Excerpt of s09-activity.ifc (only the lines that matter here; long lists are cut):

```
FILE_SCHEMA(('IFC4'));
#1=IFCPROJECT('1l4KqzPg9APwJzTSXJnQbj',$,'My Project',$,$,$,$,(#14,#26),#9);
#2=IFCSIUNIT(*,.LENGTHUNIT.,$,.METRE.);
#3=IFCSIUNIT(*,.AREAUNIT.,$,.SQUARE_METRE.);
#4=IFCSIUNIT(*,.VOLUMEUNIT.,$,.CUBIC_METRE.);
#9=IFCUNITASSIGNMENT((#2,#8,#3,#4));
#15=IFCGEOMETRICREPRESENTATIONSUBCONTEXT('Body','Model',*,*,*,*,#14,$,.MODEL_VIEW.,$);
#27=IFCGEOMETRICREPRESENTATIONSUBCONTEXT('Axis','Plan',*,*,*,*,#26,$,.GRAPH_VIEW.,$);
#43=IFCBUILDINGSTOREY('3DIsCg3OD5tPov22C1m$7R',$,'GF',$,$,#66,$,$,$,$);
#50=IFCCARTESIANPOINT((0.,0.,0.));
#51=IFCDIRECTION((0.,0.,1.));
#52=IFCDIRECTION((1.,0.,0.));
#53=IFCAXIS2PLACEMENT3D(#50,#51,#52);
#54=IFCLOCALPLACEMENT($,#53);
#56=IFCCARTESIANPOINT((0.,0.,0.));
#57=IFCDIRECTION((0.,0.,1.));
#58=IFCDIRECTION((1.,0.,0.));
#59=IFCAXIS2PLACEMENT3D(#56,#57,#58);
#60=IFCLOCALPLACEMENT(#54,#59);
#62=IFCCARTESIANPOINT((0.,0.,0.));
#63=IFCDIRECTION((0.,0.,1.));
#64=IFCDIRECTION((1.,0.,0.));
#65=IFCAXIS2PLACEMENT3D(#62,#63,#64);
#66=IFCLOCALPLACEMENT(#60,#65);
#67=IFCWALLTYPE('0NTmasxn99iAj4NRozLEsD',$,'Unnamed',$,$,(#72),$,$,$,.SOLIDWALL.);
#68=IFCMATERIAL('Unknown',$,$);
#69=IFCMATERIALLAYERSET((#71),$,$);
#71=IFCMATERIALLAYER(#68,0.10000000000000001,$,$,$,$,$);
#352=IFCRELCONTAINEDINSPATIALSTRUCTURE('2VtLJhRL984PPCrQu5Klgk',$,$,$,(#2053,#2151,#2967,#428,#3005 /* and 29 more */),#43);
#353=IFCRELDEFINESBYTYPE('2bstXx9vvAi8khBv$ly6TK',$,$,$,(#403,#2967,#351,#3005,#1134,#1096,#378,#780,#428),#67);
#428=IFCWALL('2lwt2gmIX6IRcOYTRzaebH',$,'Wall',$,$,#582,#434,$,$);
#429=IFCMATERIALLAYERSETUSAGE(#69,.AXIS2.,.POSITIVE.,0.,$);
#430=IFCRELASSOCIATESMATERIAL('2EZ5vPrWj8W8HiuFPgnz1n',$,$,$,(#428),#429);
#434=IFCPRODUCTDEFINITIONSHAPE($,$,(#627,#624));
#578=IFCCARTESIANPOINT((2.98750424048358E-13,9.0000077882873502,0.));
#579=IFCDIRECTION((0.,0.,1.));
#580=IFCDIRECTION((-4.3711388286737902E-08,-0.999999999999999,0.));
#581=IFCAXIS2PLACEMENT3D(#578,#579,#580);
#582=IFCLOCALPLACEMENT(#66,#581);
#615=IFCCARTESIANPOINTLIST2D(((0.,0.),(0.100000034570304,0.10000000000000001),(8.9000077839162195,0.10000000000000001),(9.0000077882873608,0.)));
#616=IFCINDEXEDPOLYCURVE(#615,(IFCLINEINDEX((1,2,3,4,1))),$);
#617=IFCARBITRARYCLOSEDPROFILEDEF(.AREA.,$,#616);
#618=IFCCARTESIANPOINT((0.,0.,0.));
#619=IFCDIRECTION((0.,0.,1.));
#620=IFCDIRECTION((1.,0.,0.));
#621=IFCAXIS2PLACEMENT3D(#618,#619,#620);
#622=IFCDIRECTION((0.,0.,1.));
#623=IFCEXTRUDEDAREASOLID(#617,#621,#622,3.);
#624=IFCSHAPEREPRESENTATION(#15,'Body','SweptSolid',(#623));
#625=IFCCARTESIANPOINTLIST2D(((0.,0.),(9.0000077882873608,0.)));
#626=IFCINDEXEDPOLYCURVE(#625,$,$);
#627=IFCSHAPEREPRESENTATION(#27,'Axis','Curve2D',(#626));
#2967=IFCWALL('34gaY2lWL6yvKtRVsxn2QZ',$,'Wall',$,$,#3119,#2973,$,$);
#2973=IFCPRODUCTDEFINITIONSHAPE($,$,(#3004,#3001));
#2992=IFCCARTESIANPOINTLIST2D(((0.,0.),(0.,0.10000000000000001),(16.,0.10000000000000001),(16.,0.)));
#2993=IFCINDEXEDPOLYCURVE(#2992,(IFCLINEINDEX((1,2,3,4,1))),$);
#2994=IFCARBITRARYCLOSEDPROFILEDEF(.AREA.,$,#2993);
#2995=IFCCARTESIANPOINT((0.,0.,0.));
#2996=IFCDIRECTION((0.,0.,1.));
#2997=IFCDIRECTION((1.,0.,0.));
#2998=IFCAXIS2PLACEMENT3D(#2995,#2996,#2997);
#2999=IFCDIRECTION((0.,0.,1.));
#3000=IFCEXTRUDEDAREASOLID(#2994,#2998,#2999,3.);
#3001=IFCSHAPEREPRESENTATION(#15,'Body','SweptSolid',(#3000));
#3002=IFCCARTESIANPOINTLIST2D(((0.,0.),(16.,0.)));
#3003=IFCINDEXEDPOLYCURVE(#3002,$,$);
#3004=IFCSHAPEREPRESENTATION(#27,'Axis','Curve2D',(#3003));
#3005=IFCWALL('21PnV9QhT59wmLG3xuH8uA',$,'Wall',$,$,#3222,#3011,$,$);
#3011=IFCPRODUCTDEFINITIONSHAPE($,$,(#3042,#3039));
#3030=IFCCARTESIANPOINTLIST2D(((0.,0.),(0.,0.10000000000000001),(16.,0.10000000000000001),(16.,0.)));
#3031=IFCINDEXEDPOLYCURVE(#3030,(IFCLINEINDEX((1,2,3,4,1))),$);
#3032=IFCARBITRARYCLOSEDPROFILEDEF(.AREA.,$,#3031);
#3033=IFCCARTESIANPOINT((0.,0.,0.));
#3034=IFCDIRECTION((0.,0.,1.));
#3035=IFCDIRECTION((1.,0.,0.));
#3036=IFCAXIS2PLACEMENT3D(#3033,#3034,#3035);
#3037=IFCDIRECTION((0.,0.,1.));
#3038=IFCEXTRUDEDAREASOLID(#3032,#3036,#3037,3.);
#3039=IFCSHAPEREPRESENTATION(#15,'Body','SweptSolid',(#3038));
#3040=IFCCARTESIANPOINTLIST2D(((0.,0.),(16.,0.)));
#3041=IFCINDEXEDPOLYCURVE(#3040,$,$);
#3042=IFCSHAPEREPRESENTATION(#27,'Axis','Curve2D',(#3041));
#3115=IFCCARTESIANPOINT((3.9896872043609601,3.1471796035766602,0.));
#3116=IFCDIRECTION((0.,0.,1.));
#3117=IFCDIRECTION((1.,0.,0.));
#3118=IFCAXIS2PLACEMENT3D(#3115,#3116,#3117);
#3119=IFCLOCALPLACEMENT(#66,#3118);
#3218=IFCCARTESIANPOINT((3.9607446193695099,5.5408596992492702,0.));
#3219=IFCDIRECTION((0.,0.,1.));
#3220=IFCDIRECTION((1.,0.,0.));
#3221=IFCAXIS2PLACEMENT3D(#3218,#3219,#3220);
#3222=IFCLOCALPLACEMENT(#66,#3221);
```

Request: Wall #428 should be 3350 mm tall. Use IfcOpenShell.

```python
import ifcopenshell
import ifcopenshell.geom
import ifcopenshell.util.representation
import ifcopenshell.util.shape

model = ifcopenshell.open("s09-activity.ifc")
settings = ifcopenshell.geom.settings()


def volume(element):
    """Net volume in cubic metres, openings subtracted."""
    shape = ifcopenshell.geom.create_shape(settings, element)
    return ifcopenshell.util.shape.get_volume(shape.geometry)


wall = model.by_guid("2lwt2gmIX6IRcOYTRzaebH")
before = volume(wall)

body = ifcopenshell.util.representation.get_representation(wall, "Model", "Body")
solid = body.Items[0]
old_height = solid.Depth
solid.Depth = 3.35
after = volume(wall)

print(f"height {old_height:g} -> {solid.Depth:g}, volume {before:.3f} -> {after:.3f} m3")

model.write("s09-activity_v2.ifc")
```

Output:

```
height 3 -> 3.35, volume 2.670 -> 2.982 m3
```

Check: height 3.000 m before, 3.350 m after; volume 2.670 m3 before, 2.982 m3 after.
